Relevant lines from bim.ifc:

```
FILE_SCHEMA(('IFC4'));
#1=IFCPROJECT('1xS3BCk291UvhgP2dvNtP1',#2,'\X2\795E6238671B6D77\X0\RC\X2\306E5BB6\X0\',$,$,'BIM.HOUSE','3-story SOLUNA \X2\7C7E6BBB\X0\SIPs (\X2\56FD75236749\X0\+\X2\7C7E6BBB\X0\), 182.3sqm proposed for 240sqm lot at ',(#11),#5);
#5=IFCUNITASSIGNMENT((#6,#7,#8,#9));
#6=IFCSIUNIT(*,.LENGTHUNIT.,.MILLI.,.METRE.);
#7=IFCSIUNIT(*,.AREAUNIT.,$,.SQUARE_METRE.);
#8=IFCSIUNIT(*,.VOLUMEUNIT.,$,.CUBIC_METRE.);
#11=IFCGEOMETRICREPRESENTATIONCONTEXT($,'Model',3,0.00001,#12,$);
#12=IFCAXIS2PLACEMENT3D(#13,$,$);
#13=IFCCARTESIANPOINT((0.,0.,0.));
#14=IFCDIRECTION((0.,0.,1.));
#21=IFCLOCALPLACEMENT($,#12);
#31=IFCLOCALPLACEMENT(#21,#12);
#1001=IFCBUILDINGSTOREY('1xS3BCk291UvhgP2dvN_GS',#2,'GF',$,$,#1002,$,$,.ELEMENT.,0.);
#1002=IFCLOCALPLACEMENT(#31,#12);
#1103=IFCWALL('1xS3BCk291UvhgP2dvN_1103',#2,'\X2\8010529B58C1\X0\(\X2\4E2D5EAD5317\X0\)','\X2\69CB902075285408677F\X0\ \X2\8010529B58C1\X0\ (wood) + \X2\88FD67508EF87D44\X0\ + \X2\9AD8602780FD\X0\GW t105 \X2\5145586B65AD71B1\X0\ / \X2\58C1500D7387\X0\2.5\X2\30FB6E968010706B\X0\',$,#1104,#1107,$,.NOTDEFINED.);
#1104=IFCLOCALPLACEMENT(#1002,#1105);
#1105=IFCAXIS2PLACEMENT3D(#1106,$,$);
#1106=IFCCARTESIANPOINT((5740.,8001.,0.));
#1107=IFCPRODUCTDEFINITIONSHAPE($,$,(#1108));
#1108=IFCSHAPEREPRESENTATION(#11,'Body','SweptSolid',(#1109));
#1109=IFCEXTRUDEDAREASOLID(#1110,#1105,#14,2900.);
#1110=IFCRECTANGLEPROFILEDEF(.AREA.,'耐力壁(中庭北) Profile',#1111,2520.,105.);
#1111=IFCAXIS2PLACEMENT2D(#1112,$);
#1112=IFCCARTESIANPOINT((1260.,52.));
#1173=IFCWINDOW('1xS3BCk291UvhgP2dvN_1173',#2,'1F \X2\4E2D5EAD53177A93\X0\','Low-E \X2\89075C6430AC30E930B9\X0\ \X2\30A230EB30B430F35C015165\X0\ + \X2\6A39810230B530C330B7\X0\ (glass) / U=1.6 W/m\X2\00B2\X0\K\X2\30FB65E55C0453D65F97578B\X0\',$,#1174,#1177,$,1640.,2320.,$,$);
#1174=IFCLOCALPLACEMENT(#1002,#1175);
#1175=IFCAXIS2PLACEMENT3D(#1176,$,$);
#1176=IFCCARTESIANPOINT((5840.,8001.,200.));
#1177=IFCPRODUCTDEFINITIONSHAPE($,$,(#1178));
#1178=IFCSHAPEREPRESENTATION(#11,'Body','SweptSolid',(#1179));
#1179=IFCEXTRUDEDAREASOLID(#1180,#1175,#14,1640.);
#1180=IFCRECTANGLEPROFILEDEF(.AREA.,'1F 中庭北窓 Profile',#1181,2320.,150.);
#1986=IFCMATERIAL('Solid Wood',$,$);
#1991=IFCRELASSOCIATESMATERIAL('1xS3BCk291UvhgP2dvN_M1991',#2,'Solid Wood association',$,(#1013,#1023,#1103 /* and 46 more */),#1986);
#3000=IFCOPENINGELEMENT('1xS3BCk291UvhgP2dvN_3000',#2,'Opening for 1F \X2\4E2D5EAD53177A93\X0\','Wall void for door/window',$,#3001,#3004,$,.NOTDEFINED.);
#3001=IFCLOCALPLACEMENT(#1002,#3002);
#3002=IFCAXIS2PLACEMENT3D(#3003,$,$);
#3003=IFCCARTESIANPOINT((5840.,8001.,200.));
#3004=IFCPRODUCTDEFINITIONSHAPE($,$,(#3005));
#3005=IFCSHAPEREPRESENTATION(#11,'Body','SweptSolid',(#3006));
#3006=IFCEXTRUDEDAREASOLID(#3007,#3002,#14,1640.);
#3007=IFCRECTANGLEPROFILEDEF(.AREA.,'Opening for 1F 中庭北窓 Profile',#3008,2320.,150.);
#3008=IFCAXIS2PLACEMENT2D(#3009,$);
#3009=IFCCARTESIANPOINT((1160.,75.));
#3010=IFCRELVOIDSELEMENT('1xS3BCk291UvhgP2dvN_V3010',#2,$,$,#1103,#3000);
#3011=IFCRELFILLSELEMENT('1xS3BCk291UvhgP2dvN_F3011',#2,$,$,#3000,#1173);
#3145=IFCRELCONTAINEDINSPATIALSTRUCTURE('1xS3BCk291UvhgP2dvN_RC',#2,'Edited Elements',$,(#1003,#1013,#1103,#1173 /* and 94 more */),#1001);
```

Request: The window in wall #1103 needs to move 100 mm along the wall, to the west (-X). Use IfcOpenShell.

```python
import ifcopenshell
import ifcopenshell.api.geometry
import ifcopenshell.util.placement

model = ifcopenshell.open("bim.ifc")

window = model.by_guid("1xS3BCk291UvhgP2dvN_1173")
opening = window.FillsVoids[0].RelatingOpeningElement
wall = opening.VoidsElements[0].RelatingBuildingElement

wall_matrix = ifcopenshell.util.placement.get_local_placement(wall.ObjectPlacement)
shift = wall_matrix[:3, 0] * -100.0
before = ifcopenshell.util.placement.get_local_placement(window.ObjectPlacement)[:3, 3].copy()

# The window is not placed relative to its opening, so move both.
for product in (opening, window):
    matrix = ifcopenshell.util.placement.get_local_placement(product.ObjectPlacement)
    matrix[:3, 3] += shift
    ifcopenshell.api.geometry.edit_object_placement(model, product=product, matrix=matrix, is_si=False)

after = ifcopenshell.util.placement.get_local_placement(window.ObjectPlacement)[:3, 3]
print("window moved by", (after - before).round(3) + 0.0)

model.write("bim_edited.ifc")
```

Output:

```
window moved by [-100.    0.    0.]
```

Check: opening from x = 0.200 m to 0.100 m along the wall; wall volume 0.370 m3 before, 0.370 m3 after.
